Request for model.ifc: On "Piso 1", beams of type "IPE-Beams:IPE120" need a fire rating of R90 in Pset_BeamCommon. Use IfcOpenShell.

First a look at what the model holds.

```python
import ifcopenshell
import ifcopenshell.util.element

model = ifcopenshell.open("model.ifc")
print(model.schema)
storey = next(s for s in model.by_type("IfcBuildingStorey") if s.Name == "Piso 1")
beams = [e for e in ifcopenshell.util.element.get_decomposition(storey) if e.is_a("IfcBeam")]
seen = {}
for e in beams:
    element_type = ifcopenshell.util.element.get_type(e)
    key = (element_type.Name if element_type != e and element_type else None, ifcopenshell.util.element.get_pset(e, "Pset_BeamCommon", "FireRating"))
    seen[key] = seen.get(key, 0) + 1
for (name, value), count in sorted(seen.items(), key=str):
    print(count, "x", name, "|", value)
```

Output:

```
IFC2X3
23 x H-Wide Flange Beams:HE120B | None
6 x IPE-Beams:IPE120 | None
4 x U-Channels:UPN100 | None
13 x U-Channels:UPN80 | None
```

```python
import ifcopenshell
import ifcopenshell.api.pset
import ifcopenshell.util.element

model = ifcopenshell.open("model.ifc")

storey = next(s for s in model.by_type("IfcBuildingStorey") if s.Name == "Piso 1")
beams = [e for e in ifcopenshell.util.element.get_decomposition(storey) if e.is_a("IfcBeam")]

count = 0
for e in beams:
    element_type = ifcopenshell.util.element.get_type(e)
    if element_type in (None, e) or element_type.Name != "IPE-Beams:IPE120":
        continue
    # add_pset returns the element's existing set when there is one.
    pset = ifcopenshell.api.pset.add_pset(model, product=e, name="Pset_BeamCommon")
    ifcopenshell.api.pset.edit_pset(model, pset=pset, properties={"FireRating": "R90"})
    count += 1

print(count, "beams updated")

model.write("model_rev.ifc")
```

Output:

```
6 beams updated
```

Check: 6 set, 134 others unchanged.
